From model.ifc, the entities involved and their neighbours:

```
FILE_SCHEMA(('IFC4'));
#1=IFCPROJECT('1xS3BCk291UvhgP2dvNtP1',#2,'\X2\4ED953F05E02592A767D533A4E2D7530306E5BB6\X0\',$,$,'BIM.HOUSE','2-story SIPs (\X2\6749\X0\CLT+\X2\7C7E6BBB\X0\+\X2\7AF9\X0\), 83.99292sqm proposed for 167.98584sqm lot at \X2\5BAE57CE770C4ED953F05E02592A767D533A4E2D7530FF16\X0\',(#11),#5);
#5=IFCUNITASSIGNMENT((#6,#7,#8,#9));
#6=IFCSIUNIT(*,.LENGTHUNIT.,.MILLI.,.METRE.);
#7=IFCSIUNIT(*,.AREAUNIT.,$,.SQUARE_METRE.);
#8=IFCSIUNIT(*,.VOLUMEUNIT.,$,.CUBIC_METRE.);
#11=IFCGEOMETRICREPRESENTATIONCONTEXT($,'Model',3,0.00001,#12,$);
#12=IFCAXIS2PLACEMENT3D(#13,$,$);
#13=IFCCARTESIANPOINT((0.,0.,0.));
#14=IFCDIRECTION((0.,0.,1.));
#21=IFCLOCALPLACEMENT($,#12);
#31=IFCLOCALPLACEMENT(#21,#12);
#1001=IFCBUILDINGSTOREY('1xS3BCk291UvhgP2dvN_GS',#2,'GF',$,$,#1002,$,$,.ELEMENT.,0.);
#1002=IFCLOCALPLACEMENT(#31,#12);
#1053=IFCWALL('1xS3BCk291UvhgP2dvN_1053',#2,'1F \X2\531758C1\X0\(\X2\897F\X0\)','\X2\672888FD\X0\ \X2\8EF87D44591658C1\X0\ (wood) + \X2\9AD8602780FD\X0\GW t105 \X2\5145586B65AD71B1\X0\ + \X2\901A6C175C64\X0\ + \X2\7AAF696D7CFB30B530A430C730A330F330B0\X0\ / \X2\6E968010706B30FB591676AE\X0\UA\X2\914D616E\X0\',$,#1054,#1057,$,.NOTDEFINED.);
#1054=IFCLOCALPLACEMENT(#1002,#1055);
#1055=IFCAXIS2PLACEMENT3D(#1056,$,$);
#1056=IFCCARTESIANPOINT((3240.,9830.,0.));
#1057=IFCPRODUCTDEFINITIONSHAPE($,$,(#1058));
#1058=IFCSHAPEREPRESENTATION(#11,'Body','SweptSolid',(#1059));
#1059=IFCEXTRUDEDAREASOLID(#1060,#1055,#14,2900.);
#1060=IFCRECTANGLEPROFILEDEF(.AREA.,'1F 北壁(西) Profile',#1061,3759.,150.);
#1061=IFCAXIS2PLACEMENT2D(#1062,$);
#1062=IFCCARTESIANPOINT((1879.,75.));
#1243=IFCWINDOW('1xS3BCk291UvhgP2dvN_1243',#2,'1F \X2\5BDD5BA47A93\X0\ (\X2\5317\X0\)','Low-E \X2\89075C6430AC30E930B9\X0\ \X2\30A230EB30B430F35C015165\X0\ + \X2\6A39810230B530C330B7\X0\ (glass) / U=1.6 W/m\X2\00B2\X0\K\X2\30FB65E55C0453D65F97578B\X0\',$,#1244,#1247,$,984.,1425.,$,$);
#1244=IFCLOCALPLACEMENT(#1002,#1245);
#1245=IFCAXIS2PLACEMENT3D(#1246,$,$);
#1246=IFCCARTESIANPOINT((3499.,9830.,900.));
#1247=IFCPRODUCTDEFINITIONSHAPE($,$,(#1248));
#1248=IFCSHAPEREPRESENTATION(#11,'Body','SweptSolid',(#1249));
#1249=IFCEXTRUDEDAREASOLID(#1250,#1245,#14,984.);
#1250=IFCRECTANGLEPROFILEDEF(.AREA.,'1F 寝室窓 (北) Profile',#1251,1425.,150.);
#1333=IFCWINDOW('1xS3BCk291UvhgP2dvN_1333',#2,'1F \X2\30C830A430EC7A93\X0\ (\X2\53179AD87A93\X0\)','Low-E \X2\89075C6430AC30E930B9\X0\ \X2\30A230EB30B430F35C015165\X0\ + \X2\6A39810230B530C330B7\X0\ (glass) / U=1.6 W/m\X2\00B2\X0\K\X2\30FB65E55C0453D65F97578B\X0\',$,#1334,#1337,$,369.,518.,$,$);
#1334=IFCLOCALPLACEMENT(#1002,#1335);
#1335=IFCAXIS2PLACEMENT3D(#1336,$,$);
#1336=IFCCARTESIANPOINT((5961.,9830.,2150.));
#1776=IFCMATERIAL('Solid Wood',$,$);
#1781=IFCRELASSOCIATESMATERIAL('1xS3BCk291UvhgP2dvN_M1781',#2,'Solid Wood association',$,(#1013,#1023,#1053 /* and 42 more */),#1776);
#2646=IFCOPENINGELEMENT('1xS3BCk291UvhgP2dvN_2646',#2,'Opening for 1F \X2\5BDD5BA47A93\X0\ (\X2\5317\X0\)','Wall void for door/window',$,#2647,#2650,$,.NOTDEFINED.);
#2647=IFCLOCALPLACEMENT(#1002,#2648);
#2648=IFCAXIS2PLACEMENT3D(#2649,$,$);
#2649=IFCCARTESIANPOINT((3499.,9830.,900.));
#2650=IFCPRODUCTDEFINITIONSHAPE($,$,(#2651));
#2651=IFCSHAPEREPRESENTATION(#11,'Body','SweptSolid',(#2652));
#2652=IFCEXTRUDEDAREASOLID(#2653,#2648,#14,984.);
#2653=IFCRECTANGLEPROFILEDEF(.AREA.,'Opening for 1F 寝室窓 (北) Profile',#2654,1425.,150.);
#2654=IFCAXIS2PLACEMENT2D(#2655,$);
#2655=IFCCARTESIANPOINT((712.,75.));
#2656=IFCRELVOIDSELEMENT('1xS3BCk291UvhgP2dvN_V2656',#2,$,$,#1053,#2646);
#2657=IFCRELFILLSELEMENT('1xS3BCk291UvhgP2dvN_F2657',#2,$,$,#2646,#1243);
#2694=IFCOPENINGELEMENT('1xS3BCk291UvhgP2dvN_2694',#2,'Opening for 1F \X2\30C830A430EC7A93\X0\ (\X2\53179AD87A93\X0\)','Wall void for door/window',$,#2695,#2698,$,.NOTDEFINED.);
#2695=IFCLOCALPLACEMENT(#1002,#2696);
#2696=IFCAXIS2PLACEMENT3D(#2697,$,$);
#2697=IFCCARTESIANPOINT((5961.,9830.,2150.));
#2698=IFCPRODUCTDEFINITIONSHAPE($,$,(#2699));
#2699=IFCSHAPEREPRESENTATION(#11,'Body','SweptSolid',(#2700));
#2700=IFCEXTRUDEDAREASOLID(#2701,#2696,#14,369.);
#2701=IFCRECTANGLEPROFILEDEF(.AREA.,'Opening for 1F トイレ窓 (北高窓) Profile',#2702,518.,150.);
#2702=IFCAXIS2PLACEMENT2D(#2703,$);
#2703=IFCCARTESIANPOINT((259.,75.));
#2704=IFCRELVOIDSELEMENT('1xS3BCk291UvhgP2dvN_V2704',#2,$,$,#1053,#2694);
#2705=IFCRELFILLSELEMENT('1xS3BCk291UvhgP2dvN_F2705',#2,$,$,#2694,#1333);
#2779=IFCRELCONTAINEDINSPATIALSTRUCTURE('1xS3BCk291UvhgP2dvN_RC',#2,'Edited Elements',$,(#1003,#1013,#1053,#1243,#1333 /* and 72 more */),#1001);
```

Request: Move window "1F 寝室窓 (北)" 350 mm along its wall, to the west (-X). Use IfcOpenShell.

```python
import ifcopenshell
import ifcopenshell.api.geometry
import ifcopenshell.util.placement
import ifcopenshell.util.unit

model = ifcopenshell.open("model.ifc")
unit_scale = ifcopenshell.util.unit.calculate_unit_scale(model)

window = model.by_guid("1xS3BCk291UvhgP2dvN_1243")
opening = window.FillsVoids[0].RelatingOpeningElement
wall = opening.VoidsElements[0].RelatingBuildingElement

wall_matrix = ifcopenshell.util.placement.get_local_placement(wall.ObjectPlacement)
shift = wall_matrix[:3, 0] * -0.35 / unit_scale
before = ifcopenshell.util.placement.get_local_placement(window.ObjectPlacement)[:3, 3].copy()

# The window is not placed relative to its opening, so move both.
for product in (opening, window):
    matrix = ifcopenshell.util.placement.get_local_placement(product.ObjectPlacement)
    matrix[:3, 3] += shift
    ifcopenshell.api.geometry.edit_object_placement(model, product=product, matrix=matrix, is_si=False)

after = ifcopenshell.util.placement.get_local_placement(window.ObjectPlacement)[:3, 3]
print("window moved by", (after - before).round(3) + 0.0)

model.write("model_edited.ifc")
```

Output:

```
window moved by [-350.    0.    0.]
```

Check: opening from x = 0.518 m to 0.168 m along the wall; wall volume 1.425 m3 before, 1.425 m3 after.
